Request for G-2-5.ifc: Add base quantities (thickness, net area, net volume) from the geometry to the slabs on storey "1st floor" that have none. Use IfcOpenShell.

First a look at what the model holds.

```python
import ifcopenshell
import ifcopenshell.util.element
import ifcopenshell.util.unit

model = ifcopenshell.open("G-2-5.ifc")
print(model.schema)
for unit_type in ("LENGTHUNIT", "AREAUNIT", "VOLUMEUNIT"):
    print(unit_type, ifcopenshell.util.unit.calculate_unit_scale(model, unit_type))
storey = next(s for s in model.by_type("IfcBuildingStorey") if s.Name == "1st floor")
slabs = [e for e in ifcopenshell.util.element.get_decomposition(storey) if e.is_a("IfcSlab")]
for e in sorted(slabs, key=lambda e: e.id()):
    print(e.id(), e.is_a(), e.Name, list(ifcopenshell.util.element.get_psets(e, qtos_only=True)), sep=" | ")
```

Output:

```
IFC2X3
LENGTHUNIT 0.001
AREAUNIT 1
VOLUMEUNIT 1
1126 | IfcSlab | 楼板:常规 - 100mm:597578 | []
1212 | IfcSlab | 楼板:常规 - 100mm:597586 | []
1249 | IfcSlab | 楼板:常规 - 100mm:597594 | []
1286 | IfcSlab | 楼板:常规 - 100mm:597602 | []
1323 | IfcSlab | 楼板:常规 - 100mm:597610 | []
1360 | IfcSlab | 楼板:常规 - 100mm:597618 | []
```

```python
import ifcopenshell
import ifcopenshell.api.pset
import ifcopenshell.geom
import ifcopenshell.util.element
import ifcopenshell.util.shape
import ifcopenshell.util.unit

model = ifcopenshell.open("G-2-5.ifc")
unit_scale = ifcopenshell.util.unit.calculate_unit_scale(model)
area_scale = ifcopenshell.util.unit.calculate_unit_scale(model, "AREAUNIT")
volume_scale = ifcopenshell.util.unit.calculate_unit_scale(model, "VOLUMEUNIT")
settings = ifcopenshell.geom.settings()

storey = next(s for s in model.by_type("IfcBuildingStorey") if s.Name == "1st floor")
slabs = [e for e in ifcopenshell.util.element.get_decomposition(storey) if e.is_a("IfcSlab")]

for e in sorted(slabs, key=lambda e: e.id()):
    if ifcopenshell.util.element.get_psets(e, qtos_only=True, should_inherit=False):
        continue
    # Geometry comes back in metres, in the element's own axes.
    shape = ifcopenshell.geom.create_shape(settings, e)
    values = {
        "Width": ifcopenshell.util.shape.get_z(shape.geometry) / unit_scale,
        "NetArea": ifcopenshell.util.shape.get_footprint_area(shape.geometry) / area_scale,
        "NetVolume": ifcopenshell.util.shape.get_volume(shape.geometry) / volume_scale,
    }
    qto = ifcopenshell.api.pset.add_qto(model, product=e, name="BaseQuantities")
    ifcopenshell.api.pset.edit_qto(model, qto=qto, properties=values)
    print(e.id(), {k: round(v, 3) for k, v in values.items()})

model.write("G-2-5_updated.ifc")
```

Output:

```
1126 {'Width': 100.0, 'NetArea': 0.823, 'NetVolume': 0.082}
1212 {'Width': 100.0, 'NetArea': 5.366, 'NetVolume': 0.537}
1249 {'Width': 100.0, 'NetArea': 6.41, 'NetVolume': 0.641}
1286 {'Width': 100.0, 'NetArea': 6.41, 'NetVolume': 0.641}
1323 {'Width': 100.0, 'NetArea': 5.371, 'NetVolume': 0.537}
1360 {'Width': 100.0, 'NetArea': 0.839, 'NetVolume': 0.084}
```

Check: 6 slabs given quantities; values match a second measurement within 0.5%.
